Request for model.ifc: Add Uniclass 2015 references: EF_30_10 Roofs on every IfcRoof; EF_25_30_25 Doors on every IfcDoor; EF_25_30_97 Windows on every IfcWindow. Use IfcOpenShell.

First a look at what the model holds.

```python
import ifcopenshell

model = ifcopenshell.open("model.ifc")
print(model.schema)
print("classifications:", [c.Name for c in model.by_type("IfcClassification")])
for ifc_class in ("IfcDoor", "IfcRoof", "IfcStair", "IfcWall", "IfcWindow"):
    print(ifc_class, len(model.by_type(ifc_class)))
```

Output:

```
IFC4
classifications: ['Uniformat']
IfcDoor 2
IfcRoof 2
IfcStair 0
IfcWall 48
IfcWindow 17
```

```python
import ifcopenshell
import ifcopenshell.api.classification

model = ifcopenshell.open("model.ifc")

system = ifcopenshell.api.classification.add_classification(model, classification="Uniclass 2015")

codes = {
    "IfcRoof": ("EF_30_10", "Roofs"),
    "IfcDoor": ("EF_25_30_25", "Doors"),
    "IfcWindow": ("EF_25_30_97", "Windows"),
}
for ifc_class, (code, name) in codes.items():
    products = model.by_type(ifc_class)
    ifcopenshell.api.classification.add_reference(
        model, products=products, classification=system, identification=code, name=name
    )
    print(code, len(products))

model.write("model_rev.ifc")
```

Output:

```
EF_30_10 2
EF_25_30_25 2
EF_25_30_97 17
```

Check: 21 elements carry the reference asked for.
